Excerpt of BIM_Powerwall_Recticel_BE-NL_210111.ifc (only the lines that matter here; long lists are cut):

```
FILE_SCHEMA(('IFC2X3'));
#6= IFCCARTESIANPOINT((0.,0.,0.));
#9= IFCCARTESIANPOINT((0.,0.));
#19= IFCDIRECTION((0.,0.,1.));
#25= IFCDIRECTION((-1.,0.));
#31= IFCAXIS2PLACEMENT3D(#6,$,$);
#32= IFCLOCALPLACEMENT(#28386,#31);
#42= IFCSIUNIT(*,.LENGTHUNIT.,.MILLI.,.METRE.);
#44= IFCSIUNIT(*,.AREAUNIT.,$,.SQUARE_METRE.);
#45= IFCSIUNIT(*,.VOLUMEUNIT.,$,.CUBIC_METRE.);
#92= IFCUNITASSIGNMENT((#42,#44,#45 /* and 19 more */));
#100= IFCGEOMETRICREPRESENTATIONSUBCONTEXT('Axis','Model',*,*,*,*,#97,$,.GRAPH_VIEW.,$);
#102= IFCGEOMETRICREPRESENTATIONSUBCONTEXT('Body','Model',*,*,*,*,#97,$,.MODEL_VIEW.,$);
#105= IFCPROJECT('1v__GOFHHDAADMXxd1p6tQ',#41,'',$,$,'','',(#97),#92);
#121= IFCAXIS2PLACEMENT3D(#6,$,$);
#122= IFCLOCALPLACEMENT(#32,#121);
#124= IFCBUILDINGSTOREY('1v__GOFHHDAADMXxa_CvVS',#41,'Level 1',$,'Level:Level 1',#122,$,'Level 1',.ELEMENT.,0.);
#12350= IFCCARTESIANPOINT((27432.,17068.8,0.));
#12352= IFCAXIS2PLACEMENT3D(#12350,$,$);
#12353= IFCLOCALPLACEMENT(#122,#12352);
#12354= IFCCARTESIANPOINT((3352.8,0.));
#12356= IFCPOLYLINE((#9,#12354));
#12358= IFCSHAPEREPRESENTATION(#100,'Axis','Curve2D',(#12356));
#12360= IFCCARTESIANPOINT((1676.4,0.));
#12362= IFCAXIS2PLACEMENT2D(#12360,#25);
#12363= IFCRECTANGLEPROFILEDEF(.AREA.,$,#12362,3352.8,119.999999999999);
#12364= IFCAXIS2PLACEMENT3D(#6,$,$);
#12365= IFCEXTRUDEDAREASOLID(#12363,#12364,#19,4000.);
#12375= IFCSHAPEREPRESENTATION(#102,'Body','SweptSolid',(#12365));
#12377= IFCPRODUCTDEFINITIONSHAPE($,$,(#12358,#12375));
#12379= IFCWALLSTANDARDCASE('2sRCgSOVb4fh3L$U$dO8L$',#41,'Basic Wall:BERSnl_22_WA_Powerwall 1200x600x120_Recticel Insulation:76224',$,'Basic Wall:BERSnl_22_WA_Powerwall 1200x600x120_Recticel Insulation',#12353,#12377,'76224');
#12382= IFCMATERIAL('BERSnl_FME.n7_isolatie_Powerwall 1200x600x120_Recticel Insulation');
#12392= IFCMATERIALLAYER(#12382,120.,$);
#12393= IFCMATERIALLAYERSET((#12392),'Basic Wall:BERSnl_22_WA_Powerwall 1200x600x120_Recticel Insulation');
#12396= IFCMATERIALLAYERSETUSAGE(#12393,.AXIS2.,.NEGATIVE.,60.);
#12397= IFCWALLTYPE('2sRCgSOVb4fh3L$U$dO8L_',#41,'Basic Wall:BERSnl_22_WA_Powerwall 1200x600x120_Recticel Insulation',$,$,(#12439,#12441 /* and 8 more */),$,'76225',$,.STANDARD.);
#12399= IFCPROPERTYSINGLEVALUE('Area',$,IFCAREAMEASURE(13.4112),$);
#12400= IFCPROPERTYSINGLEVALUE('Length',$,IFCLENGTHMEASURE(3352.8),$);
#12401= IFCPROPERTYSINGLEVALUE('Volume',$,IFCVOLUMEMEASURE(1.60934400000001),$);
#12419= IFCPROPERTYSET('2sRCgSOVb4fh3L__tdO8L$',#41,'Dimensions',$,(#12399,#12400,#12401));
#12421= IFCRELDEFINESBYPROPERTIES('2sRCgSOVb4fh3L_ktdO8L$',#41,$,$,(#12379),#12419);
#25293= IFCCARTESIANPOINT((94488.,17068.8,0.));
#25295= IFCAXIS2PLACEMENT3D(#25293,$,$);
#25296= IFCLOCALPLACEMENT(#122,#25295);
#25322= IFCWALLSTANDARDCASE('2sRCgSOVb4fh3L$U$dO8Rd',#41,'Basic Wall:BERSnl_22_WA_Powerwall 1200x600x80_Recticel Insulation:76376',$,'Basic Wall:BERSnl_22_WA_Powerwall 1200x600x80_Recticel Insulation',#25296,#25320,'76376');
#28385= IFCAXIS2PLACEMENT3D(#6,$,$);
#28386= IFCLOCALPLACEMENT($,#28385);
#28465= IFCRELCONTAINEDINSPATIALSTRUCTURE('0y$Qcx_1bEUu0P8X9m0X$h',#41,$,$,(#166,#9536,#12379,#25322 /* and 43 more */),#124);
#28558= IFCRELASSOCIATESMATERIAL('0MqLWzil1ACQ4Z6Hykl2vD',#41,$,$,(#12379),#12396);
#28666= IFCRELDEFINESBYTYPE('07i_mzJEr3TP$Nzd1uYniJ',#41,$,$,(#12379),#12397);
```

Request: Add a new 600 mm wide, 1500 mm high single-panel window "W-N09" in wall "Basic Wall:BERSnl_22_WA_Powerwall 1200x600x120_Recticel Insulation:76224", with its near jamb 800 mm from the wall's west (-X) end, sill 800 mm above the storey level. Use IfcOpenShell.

```python
import numpy as np
import ifcopenshell
import ifcopenshell.api.feature
import ifcopenshell.api.geometry
import ifcopenshell.api.pset
import ifcopenshell.api.root
import ifcopenshell.api.spatial
import ifcopenshell.api.type
import ifcopenshell.geom
import ifcopenshell.util.element
import ifcopenshell.util.placement
import ifcopenshell.util.representation
import ifcopenshell.util.shape
import ifcopenshell.util.unit

model = ifcopenshell.open("BIM_Powerwall_Recticel_BE-NL_210111.ifc")
unit_scale = ifcopenshell.util.unit.calculate_unit_scale(model)
area_scale = ifcopenshell.util.unit.calculate_unit_scale(model, "AREAUNIT")
volume_scale = ifcopenshell.util.unit.calculate_unit_scale(model, "VOLUMEUNIT")
settings = ifcopenshell.geom.settings()


def volume(element):
    """Net volume in cubic metres, openings subtracted."""
    shape = ifcopenshell.geom.create_shape(settings, element)
    return ifcopenshell.util.shape.get_volume(shape.geometry)


wall = model.by_guid("2sRCgSOVb4fh3L$U$dO8L$")
storey = ifcopenshell.util.element.get_container(wall, ifc_class="IfcBuildingStorey")
context = ifcopenshell.util.representation.get_context(model, "Model", "Body", "MODEL_VIEW")
before = volume(wall)

width, height, from_end, sill = 0.6, 1.5, 0.8, 0.8  # metres

# The wall runs along its own X axis, and the end named is its -X end.
wall_shape = ifcopenshell.geom.create_shape(settings, wall)
x, y, z = ifcopenshell.util.shape.get_vertices(wall_shape.geometry).T
start = x.min() + from_end
face, thickness = float(y.min()), float(y.max() - y.min())
wall_matrix = ifcopenshell.util.placement.get_local_placement(wall.ObjectPlacement)
level = ifcopenshell.util.placement.get_local_placement(storey.ObjectPlacement)[2, 3]


def in_wall(x, y):
    """Placement at x, y metres in the wall's axes, at sill height."""
    matrix = wall_matrix.copy()
    matrix[:, 3] = wall_matrix @ np.array([x / unit_scale, y / unit_scale, 0.0, 1.0])
    matrix[2, 3] = level + sill / unit_scale
    return matrix


# Opening: a box that overshoots both wall faces by 50 mm.
opening = ifcopenshell.api.root.create_entity(model, ifc_class="IfcOpeningElement")
box = ifcopenshell.api.geometry.add_wall_representation(
    model, context=context, length=width, height=height, thickness=thickness + 0.1
)
ifcopenshell.api.geometry.assign_representation(model, product=opening, representation=box)
ifcopenshell.api.geometry.edit_object_placement(model, product=opening, matrix=in_wall(start, face - 0.05), is_si=False)
ifcopenshell.api.feature.add_feature(model, feature=opening, element=wall)

window = ifcopenshell.api.root.create_entity(model, ifc_class="IfcWindow", name="W-N09")
window.OverallWidth, window.OverallHeight = width / unit_scale, height / unit_scale
body = ifcopenshell.api.geometry.add_window_representation(
    model,
    context=context,
    overall_width=window.OverallWidth,
    overall_height=window.OverallHeight,
    partition_type="SINGLE_PANEL",
)
ifcopenshell.api.geometry.assign_representation(model, product=window, representation=body)
ifcopenshell.api.spatial.assign_container(model, products=[window], relating_structure=storey)
fills = ifcopenshell.api.feature.add_filling(model, opening=opening, element=window)
fills.OwnerHistory = window.OwnerHistory  # required in IFC2X3

# IFC2X3 keeps the operation on the window style.
style = ifcopenshell.api.root.create_entity(model, ifc_class="IfcWindowStyle", name="W-N09")
style.OperationType, style.ConstructionType = "SINGLE_PANEL", "NOTDEFINED"
style.ParameterTakesPrecedence = style.Sizeable = False
ifcopenshell.api.type.assign_type(model, related_objects=[window], relating_type=style)

# Centre the window in the wall's thickness.
ifcopenshell.api.geometry.edit_object_placement(model, product=window, matrix=in_wall(start, face), is_si=False)
window_shape = ifcopenshell.geom.create_shape(settings, window)
depth = ifcopenshell.util.shape.get_vertices(window_shape.geometry)[:, 1]
offset = face + thickness / 2 - (depth.min() + depth.max()) / 2
ifcopenshell.api.geometry.edit_object_placement(model, product=window, matrix=in_wall(start, offset), is_si=False)

after = volume(wall)

# Update the wall's stored quantities.
pset = model.by_id(ifcopenshell.util.element.get_pset(wall, "Dimensions", should_inherit=False)["id"])
ifcopenshell.api.pset.edit_pset(model, pset=pset, properties={
    "Area": model.create_entity("IfcAreaMeasure", after / thickness / area_scale),
    "Volume": model.create_entity("IfcVolumeMeasure", after / volume_scale),
})

print(f"wall volume {before:.3f} -> {after:.3f} m3")

model.write("BIM_Powerwall_Recticel_BE-NL_210111_rev.ifc")
```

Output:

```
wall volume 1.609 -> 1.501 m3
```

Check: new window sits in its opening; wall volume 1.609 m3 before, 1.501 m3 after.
